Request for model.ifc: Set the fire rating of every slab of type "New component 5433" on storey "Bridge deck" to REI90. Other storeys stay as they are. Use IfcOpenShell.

First a look at what the model holds.

```python
import ifcopenshell
import ifcopenshell.util.element

model = ifcopenshell.open("model.ifc")
print(model.schema)
storey = next(s for s in model.by_type("IfcBuildingStorey") if s.Name == "Bridge deck")
slabs = [e for e in ifcopenshell.util.element.get_decomposition(storey) if e.is_a("IfcSlab")]
seen = {}
for e in slabs:
    element_type = ifcopenshell.util.element.get_type(e)
    key = (element_type.Name if element_type != e and element_type else None, ifcopenshell.util.element.get_pset(e, "Pset_SlabCommon", "FireRating"))
    seen[key] = seen.get(key, 0) + 1
for (name, value), count in sorted(seen.items(), key=str):
    print(count, "x", name, "|", value)
```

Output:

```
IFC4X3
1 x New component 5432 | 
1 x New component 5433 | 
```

```python
import ifcopenshell
import ifcopenshell.api.pset
import ifcopenshell.util.element

model = ifcopenshell.open("model.ifc")

storey = next(s for s in model.by_type("IfcBuildingStorey") if s.Name == "Bridge deck")
slabs = [e for e in ifcopenshell.util.element.get_decomposition(storey) if e.is_a("IfcSlab")]

count = 0
for e in slabs:
    element_type = ifcopenshell.util.element.get_type(e)
    if element_type in (None, e) or element_type.Name != "New component 5433":
        continue
    # add_pset returns the element's existing set when there is one.
    pset = ifcopenshell.api.pset.add_pset(model, product=e, name="Pset_SlabCommon")
    ifcopenshell.api.pset.edit_pset(model, pset=pset, properties={"FireRating": "REI90"})
    count += 1

print(count, "slabs updated")

model.write("model-out.ifc")
```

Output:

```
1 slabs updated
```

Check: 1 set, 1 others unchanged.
